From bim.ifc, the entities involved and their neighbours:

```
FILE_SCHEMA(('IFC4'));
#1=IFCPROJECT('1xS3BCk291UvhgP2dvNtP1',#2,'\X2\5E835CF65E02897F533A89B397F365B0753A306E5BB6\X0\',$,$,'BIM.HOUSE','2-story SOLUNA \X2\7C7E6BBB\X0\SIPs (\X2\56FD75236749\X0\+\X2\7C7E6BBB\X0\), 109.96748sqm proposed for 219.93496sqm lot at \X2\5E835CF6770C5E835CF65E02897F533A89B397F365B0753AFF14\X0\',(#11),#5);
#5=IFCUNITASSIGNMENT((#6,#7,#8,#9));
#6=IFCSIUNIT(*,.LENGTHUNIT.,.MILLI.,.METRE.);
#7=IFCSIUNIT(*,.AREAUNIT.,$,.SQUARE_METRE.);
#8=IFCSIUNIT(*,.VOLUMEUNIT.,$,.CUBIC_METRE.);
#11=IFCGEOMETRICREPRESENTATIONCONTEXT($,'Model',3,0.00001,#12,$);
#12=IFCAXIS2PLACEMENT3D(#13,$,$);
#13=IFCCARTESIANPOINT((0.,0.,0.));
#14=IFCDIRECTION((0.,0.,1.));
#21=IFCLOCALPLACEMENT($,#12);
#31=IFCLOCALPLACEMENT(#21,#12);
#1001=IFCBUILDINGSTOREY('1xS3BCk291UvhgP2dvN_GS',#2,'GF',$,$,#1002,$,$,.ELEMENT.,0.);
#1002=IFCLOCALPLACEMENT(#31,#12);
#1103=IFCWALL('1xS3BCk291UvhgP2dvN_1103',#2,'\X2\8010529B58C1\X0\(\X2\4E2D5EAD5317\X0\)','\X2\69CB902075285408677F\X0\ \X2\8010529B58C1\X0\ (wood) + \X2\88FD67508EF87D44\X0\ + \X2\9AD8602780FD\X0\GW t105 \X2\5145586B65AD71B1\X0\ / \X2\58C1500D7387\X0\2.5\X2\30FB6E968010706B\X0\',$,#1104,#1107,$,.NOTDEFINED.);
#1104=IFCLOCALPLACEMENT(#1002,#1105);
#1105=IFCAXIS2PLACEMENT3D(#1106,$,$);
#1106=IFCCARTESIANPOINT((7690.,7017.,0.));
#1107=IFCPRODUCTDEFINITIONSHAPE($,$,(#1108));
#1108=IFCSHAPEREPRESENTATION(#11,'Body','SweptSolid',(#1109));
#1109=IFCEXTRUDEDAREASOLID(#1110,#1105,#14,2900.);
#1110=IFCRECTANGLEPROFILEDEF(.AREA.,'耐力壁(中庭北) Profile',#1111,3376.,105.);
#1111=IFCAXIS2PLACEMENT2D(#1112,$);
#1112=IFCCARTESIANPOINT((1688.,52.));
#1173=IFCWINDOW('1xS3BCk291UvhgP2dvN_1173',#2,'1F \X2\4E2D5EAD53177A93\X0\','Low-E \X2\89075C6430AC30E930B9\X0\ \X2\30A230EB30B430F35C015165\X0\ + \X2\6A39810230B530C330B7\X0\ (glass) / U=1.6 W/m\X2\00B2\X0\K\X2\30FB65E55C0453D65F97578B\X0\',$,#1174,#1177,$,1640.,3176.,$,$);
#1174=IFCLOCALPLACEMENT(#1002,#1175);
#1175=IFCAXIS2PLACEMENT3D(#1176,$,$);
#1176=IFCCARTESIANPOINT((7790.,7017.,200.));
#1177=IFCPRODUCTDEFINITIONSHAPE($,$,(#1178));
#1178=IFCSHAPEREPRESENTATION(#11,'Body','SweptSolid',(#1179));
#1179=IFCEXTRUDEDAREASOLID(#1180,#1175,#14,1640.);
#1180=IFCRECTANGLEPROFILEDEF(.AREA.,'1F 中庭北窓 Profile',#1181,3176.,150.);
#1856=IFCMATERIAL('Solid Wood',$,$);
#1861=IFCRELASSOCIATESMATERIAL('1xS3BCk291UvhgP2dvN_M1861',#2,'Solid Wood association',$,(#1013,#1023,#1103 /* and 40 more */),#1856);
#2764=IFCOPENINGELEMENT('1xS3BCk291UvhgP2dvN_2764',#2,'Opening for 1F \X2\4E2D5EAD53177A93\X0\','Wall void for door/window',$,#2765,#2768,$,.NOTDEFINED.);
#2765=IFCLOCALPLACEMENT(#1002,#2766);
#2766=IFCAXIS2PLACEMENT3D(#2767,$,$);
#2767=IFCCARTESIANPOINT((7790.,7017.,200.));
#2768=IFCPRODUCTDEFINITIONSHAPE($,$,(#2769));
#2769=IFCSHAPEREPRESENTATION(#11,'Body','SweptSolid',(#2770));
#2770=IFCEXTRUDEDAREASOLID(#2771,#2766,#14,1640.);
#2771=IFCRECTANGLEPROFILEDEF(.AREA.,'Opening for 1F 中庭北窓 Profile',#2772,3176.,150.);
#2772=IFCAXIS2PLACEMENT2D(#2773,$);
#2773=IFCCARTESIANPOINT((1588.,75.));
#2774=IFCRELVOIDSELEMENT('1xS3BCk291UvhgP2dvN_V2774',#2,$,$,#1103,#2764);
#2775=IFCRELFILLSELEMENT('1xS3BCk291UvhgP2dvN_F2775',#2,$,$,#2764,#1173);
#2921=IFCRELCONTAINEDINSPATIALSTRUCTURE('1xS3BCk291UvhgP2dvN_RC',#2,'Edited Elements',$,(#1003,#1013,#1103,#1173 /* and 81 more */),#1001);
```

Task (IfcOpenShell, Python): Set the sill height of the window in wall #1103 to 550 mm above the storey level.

```python
import numpy as np
import ifcopenshell
import ifcopenshell.api.geometry
import ifcopenshell.geom
import ifcopenshell.util.element
import ifcopenshell.util.placement
import ifcopenshell.util.shape
import ifcopenshell.util.unit

model = ifcopenshell.open("bim.ifc")
unit_scale = ifcopenshell.util.unit.calculate_unit_scale(model)

window = model.by_guid("1xS3BCk291UvhgP2dvN_1173")
opening = window.FillsVoids[0].RelatingOpeningElement
storey = ifcopenshell.util.element.get_container(window, ifc_class="IfcBuildingStorey")
level = ifcopenshell.util.placement.get_local_placement(storey.ObjectPlacement)[2, 3]

# The opening's origin need not be at the sill, so measure its lowest point.
shape = ifcopenshell.geom.create_shape(ifcopenshell.geom.settings(), opening)
bottom = ifcopenshell.util.shape.get_shape_bottom_elevation(shape, shape.geometry) / unit_scale
dz = level + 0.55 / unit_scale - bottom

shift = np.array([0.0, 0.0, dz])
# The window is not placed relative to its opening, so move both.
for product in (opening, window):
    matrix = ifcopenshell.util.placement.get_local_placement(product.ObjectPlacement)
    matrix[:3, 3] += shift
    ifcopenshell.api.geometry.edit_object_placement(model, product=product, matrix=matrix, is_si=False)

print(f"moved by {dz * unit_scale:+.3f} m")

model.write("bim-out.ifc")
```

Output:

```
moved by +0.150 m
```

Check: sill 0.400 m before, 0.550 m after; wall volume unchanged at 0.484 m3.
